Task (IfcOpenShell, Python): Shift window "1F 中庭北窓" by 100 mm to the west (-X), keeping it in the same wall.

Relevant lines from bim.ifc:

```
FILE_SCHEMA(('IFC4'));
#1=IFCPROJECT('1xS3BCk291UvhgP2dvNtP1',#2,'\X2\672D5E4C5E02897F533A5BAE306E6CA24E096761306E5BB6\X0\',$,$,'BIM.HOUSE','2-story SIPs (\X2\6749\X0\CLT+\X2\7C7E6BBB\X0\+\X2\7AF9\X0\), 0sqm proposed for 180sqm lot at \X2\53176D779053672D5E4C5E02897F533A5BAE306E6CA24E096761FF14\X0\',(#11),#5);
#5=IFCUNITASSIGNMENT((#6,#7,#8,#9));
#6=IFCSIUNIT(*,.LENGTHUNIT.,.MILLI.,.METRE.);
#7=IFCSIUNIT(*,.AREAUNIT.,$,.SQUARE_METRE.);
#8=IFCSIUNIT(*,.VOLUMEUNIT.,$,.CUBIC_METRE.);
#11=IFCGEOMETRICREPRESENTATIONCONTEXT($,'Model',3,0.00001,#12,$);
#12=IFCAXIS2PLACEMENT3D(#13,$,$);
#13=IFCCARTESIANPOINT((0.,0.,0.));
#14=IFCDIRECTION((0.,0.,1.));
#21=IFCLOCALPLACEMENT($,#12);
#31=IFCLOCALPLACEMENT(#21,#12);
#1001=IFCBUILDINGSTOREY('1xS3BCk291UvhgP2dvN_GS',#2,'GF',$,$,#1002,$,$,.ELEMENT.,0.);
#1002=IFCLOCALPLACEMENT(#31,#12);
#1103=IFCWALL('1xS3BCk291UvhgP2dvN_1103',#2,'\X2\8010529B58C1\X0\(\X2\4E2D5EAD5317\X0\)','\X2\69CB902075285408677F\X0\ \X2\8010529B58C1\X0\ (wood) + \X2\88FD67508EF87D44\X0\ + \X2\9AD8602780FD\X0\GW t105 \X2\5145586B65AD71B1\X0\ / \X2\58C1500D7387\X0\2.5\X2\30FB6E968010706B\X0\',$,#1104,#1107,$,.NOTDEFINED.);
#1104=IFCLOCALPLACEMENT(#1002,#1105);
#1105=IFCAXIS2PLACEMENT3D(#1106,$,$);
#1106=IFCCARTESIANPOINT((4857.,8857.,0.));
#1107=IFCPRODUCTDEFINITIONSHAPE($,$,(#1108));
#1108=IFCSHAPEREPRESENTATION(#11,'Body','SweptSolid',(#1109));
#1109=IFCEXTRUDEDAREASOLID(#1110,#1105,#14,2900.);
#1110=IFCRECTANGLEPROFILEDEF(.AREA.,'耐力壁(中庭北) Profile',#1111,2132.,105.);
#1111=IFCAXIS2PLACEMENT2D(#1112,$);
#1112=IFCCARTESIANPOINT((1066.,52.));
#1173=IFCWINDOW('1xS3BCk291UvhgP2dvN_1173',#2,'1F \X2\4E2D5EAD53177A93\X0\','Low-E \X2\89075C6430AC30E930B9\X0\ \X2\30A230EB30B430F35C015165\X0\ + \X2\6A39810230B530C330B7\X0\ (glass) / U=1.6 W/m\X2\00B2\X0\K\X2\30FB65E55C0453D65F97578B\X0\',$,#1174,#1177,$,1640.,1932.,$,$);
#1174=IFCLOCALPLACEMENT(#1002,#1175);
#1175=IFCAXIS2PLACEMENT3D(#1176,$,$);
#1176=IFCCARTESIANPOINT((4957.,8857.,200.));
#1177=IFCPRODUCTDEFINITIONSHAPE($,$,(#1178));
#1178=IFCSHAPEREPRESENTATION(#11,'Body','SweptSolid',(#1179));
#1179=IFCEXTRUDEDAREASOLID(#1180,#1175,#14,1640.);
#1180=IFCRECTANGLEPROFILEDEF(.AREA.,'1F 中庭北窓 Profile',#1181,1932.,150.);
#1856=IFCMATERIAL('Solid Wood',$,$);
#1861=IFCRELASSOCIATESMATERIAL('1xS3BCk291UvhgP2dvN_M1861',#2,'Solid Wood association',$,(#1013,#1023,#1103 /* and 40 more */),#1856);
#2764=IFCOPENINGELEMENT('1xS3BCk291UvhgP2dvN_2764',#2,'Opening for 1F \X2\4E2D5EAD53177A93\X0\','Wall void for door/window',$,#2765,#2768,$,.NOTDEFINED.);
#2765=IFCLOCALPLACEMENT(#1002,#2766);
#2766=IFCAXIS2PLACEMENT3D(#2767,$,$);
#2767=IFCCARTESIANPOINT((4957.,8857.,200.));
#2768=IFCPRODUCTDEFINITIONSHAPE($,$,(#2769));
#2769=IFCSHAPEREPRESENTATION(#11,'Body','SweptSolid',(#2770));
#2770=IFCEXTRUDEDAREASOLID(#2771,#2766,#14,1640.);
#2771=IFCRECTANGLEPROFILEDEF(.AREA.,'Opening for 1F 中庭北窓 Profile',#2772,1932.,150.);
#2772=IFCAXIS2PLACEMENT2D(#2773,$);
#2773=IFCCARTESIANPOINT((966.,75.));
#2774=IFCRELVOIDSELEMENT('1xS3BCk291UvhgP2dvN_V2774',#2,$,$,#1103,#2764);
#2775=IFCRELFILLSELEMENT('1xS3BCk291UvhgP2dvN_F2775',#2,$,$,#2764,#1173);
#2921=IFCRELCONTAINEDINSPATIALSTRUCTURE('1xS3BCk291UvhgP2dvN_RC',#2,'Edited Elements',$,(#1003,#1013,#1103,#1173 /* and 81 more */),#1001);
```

```python
import ifcopenshell
import ifcopenshell.api.geometry
import ifcopenshell.util.placement
import ifcopenshell.util.unit

model = ifcopenshell.open("bim.ifc")
unit_scale = ifcopenshell.util.unit.calculate_unit_scale(model)

window = model.by_id(1173)
opening = window.FillsVoids[0].RelatingOpeningElement
wall = opening.VoidsElements[0].RelatingBuildingElement

wall_matrix = ifcopenshell.util.placement.get_local_placement(wall.ObjectPlacement)
shift = wall_matrix[:3, 0] * -0.1 / unit_scale
before = ifcopenshell.util.placement.get_local_placement(window.ObjectPlacement)[:3, 3].copy()

# The window is not placed relative to its opening, so move both.
for product in (opening, window):
    matrix = ifcopenshell.util.placement.get_local_placement(product.ObjectPlacement)
    matrix[:3, 3] += shift
    ifcopenshell.api.geometry.edit_object_placement(model, product=product, matrix=matrix, is_si=False)

after = ifcopenshell.util.placement.get_local_placement(window.ObjectPlacement)[:3, 3]
print("window moved by", (after - before).round(3) + 0.0)

model.write("bim-out.ifc")
```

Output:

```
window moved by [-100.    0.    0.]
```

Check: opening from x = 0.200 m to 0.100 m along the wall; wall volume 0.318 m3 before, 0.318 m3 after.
